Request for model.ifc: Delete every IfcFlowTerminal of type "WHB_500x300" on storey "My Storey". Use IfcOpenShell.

First a look at what the model holds.

```python
import ifcopenshell
import ifcopenshell.util.element

model = ifcopenshell.open("model.ifc")
print(model.schema)
storey = next(s for s in model.by_type("IfcBuildingStorey") if s.Name == "My Storey")
terminals = [e for e in ifcopenshell.util.element.get_decomposition(storey) if e.is_a("IfcFlowTerminal")]
seen = {}
for e in terminals:
    element_type = ifcopenshell.util.element.get_type(e)
    name = element_type.Name if element_type not in (None, e) else None
    seen[name] = seen.get(name, 0) + 1
for name, count in sorted(seen.items(), key=str):
    print(count, "x", name)
```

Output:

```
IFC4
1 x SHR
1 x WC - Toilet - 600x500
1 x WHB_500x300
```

```python
import ifcopenshell
import ifcopenshell.api.root
import ifcopenshell.util.element

model = ifcopenshell.open("model.ifc")

storey = next(s for s in model.by_type("IfcBuildingStorey") if s.Name == "My Storey")
terminals = [e for e in ifcopenshell.util.element.get_decomposition(storey) if e.is_a("IfcFlowTerminal")]
targets = [e for e in terminals if (t := ifcopenshell.util.element.get_type(e)) not in (None, e) and t.Name == "WHB_500x300"]

for e in targets:
    ifcopenshell.api.root.remove_product(model, product=e)
print(len(targets), "removed")

model.write("model_v2.ifc")
```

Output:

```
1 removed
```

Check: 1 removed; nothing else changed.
